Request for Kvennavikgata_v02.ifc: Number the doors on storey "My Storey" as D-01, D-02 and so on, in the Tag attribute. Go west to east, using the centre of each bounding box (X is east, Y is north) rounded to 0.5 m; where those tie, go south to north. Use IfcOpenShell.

First a look at what the model holds.

```python
import ifcopenshell
import ifcopenshell.util.element
import ifcopenshell.util.placement

model = ifcopenshell.open("Kvennavikgata_v02.ifc")
print(model.schema)
storey = next(s for s in model.by_type("IfcBuildingStorey") if s.Name == "My Storey")
doors = [e for e in ifcopenshell.util.element.get_decomposition(storey) if e.is_a("IfcDoor")]
for e in sorted(doors, key=lambda e: e.id()):
    origin = ifcopenshell.util.placement.get_local_placement(e.ObjectPlacement)[:3, 3]
    print(e.id(), e.Tag, e.Name, origin.round(2) + 0.0, sep=" | ")
```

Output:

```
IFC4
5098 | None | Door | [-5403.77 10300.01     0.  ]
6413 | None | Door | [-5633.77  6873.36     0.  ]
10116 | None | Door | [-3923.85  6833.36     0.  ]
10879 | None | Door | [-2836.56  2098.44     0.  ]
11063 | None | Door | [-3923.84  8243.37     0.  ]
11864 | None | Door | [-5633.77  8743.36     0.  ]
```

```python
import ifcopenshell
import ifcopenshell.geom
import ifcopenshell.util.element
import ifcopenshell.util.shape

model = ifcopenshell.open("Kvennavikgata_v02.ifc")
settings = ifcopenshell.geom.settings()
settings.set("use-world-coords", True)


def centre(element):
    shape = ifcopenshell.geom.create_shape(settings, element)
    return ifcopenshell.util.shape.get_bbox_centroid(shape.geometry)


storey = next(s for s in model.by_type("IfcBuildingStorey") if s.Name == "My Storey")
doors = [e for e in ifcopenshell.util.element.get_decomposition(storey) if e.is_a("IfcDoor")]

# Insertion points can sit at a corner or the storey origin, so sort by the geometry (in metres).
centres = {e: centre(e) for e in doors}
doors.sort(key=lambda e: (round(centres[e][0] / 0.5), centres[e][1]))

for i, e in enumerate(doors, start=1):
    number = f"D-{i:02d}"
    e.Tag = number
    print(e.id(), number)

model.write("Kvennavikgata_v02_v2.ifc")
```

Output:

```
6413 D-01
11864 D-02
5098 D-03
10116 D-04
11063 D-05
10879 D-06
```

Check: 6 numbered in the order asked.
